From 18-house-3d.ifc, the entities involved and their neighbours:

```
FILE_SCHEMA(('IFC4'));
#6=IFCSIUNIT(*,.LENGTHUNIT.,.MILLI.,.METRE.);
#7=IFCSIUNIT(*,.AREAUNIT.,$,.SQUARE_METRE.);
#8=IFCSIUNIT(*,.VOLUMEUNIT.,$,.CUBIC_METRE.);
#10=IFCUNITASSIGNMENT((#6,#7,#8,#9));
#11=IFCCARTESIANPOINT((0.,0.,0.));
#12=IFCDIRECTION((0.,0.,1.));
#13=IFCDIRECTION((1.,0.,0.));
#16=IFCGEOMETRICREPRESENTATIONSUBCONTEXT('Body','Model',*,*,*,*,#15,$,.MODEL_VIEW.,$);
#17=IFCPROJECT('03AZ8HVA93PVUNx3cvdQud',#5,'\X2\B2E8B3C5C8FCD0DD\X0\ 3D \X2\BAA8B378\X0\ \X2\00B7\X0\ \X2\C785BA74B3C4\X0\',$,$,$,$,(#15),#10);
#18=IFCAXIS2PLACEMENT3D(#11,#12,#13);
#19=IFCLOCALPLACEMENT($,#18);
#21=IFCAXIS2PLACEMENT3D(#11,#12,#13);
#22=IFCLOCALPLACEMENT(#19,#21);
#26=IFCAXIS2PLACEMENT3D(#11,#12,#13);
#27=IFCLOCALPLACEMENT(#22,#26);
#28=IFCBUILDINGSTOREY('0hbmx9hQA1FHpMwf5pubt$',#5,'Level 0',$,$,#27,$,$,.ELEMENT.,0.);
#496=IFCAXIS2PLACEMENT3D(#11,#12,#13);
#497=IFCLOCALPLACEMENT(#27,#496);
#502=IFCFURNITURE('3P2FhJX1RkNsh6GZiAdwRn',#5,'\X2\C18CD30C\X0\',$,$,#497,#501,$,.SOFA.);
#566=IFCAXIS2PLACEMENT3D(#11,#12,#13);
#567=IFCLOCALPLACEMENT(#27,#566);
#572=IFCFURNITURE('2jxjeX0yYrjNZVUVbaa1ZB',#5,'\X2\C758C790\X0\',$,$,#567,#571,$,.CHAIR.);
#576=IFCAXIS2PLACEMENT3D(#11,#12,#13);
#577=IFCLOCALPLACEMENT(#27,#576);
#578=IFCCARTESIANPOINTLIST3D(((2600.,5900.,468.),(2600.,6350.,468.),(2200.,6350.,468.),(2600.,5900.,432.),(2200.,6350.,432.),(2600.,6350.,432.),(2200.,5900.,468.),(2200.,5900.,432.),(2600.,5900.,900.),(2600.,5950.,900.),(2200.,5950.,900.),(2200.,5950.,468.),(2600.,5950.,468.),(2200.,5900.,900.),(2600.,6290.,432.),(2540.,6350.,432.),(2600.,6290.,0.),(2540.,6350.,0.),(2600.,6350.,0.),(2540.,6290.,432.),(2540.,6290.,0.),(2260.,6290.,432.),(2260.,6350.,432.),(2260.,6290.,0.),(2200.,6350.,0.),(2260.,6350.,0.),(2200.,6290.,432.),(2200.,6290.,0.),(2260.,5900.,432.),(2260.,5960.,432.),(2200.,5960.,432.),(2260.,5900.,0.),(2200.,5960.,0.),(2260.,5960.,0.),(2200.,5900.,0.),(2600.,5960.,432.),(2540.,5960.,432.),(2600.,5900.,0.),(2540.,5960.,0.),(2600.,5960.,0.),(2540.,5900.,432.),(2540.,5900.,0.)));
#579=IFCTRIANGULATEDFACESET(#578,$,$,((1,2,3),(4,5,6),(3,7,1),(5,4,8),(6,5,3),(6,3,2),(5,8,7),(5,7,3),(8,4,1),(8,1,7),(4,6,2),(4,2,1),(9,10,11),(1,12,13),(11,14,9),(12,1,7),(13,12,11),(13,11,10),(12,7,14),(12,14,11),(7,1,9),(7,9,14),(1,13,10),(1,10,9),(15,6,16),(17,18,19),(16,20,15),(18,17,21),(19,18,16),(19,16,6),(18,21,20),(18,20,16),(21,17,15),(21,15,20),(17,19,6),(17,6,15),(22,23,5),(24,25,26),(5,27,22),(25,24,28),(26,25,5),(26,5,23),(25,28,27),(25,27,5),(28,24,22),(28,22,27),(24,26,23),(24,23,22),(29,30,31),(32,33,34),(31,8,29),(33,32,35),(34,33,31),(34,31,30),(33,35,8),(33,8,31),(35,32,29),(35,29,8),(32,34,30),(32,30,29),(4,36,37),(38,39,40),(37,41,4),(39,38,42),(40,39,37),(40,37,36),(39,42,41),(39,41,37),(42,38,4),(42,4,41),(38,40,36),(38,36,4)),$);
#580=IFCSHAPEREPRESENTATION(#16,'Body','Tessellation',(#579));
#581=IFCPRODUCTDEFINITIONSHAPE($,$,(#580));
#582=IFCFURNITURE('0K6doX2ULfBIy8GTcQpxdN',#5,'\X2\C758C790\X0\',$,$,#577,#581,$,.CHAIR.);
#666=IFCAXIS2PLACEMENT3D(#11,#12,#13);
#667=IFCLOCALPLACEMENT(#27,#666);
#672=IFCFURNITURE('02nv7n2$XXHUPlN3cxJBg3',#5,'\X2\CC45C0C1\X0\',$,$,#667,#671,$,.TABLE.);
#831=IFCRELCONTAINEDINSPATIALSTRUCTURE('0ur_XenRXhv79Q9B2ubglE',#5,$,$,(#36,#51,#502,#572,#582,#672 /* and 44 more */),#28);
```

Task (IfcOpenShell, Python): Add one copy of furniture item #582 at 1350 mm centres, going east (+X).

```python
import numpy as np
import ifcopenshell
import ifcopenshell.api.geometry
import ifcopenshell.api.root
import ifcopenshell.util.element
import ifcopenshell.util.placement

model = ifcopenshell.open("18-house-3d.ifc")


def reuse_history(source, copy):
    """copy_class also copies each property set's owner history, people and application; keep the originals."""
    for rel in copy.IsDefinedBy:
        if rel.is_a("IfcRelDefinesByProperties") and (history := rel.RelatingPropertyDefinition.OwnerHistory):
            rel.RelatingPropertyDefinition.OwnerHistory = source.OwnerHistory
            ifcopenshell.util.element.remove_deep2(model, history)


source = model.by_guid("0K6doX2ULfBIy8GTcQpxdN")
base = ifcopenshell.util.placement.get_local_placement(source.ObjectPlacement)
step = np.array([1.0, 0.0, 0.0]) * 1350.0

for i in range(1, 2):
    copy = ifcopenshell.api.root.copy_class(model, product=source)
    copy.Representation = ifcopenshell.util.element.copy_deep(
        model, source.Representation, exclude=["IfcGeometricRepresentationContext", "IfcRepresentationMap"]
    )
    reuse_history(source, copy)
    matrix = base.copy()
    matrix[:3, 3] += i * step
    print("added at", matrix[:3, 3].round(3) + 0.0)
    ifcopenshell.api.geometry.edit_object_placement(model, product=copy, matrix=matrix, is_si=False)

model.write("18-house-3d_rev.ifc")
```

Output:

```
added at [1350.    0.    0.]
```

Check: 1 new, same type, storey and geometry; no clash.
